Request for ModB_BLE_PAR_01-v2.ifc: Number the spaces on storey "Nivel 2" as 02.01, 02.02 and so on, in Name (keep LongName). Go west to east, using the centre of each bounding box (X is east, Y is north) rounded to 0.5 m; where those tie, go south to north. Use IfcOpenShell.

First a look at what the model holds.

```python
import ifcopenshell
import ifcopenshell.util.element
import ifcopenshell.util.placement

model = ifcopenshell.open("ModB_BLE_PAR_01-v2.ifc")
print(model.schema)
storey = next(s for s in model.by_type("IfcBuildingStorey") if s.Name == "Nivel 2")
spaces = [e for e in ifcopenshell.util.element.get_decomposition(storey) if e.is_a("IfcSpace")]
for e in sorted(spaces, key=lambda e: e.id()):
    origin = ifcopenshell.util.placement.get_local_placement(e.ObjectPlacement)[:3, 3]
    print(e.id(), e.Name, e.LongName, origin.round(2) + 0.0, sep=" | ")
```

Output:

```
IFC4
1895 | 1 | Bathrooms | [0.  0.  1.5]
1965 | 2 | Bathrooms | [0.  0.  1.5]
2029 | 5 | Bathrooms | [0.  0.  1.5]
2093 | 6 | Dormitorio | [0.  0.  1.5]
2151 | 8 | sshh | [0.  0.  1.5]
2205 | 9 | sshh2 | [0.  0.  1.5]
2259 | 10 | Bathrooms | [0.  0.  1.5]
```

```python
import ifcopenshell
import ifcopenshell.geom
import ifcopenshell.util.element
import ifcopenshell.util.shape

model = ifcopenshell.open("ModB_BLE_PAR_01-v2.ifc")
settings = ifcopenshell.geom.settings()
settings.set("use-world-coords", True)


def centre(element):
    shape = ifcopenshell.geom.create_shape(settings, element)
    return ifcopenshell.util.shape.get_bbox_centroid(shape.geometry)


storey = next(s for s in model.by_type("IfcBuildingStorey") if s.Name == "Nivel 2")
spaces = [e for e in ifcopenshell.util.element.get_decomposition(storey) if e.is_a("IfcSpace")]

# Insertion points can sit at a corner or the storey origin, so sort by the geometry (in metres).
centres = {e: centre(e) for e in spaces}
spaces.sort(key=lambda e: (round(centres[e][0] / 0.5), centres[e][1]))

for i, e in enumerate(spaces, start=1):
    number = f"02.{i:02d}"
    e.Name = number
    print(e.id(), number)

model.write("ModB_BLE_PAR_01-v2_updated.ifc")
```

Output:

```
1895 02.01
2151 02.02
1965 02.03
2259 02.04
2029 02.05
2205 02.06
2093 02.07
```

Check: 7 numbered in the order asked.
